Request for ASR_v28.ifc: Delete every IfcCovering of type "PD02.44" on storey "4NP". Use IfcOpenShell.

First a look at what the model holds.

```python
import ifcopenshell
import ifcopenshell.util.element

model = ifcopenshell.open("ASR_v28.ifc")
print(model.schema)
storey = next(s for s in model.by_type("IfcBuildingStorey") if s.Name == "4NP")
coverings = [e for e in ifcopenshell.util.element.get_decomposition(storey) if e.is_a("IfcCovering")]
seen = {}
for e in coverings:
    element_type = ifcopenshell.util.element.get_type(e)
    name = element_type.Name if element_type not in (None, e) else None
    seen[name] = seen.get(name, 0) + 1
for name, count in sorted(seen.items(), key=str):
    print(count, "x", name)
```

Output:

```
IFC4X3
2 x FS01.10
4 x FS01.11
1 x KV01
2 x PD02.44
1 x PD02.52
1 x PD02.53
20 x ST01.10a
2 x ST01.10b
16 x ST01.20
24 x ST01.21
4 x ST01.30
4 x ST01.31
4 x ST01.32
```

```python
import ifcopenshell
import ifcopenshell.api.root
import ifcopenshell.util.element

model = ifcopenshell.open("ASR_v28.ifc")

storey = next(s for s in model.by_type("IfcBuildingStorey") if s.Name == "4NP")
coverings = [e for e in ifcopenshell.util.element.get_decomposition(storey) if e.is_a("IfcCovering")]
targets = [e for e in coverings if (t := ifcopenshell.util.element.get_type(e)) not in (None, e) and t.Name == "PD02.44"]

for e in targets:
    ifcopenshell.api.root.remove_product(model, product=e)
print(len(targets), "removed")

model.write("ASR_v28_rev.ifc")
```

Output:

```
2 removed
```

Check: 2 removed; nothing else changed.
